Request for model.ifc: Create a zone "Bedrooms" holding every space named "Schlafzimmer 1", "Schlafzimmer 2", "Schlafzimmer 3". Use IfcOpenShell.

First a look at what the model holds.

```python
import ifcopenshell

model = ifcopenshell.open("model.ifc")
print(model.schema)
seen = {}
for space in model.by_type("IfcSpace"):
    seen[space.LongName] = seen.get(space.LongName, 0) + 1
for name, count in sorted(seen.items(), key=str):
    print(count, "x", name)
print("zones:", [z.Name for z in model.by_type("IfcZone")][:20])
```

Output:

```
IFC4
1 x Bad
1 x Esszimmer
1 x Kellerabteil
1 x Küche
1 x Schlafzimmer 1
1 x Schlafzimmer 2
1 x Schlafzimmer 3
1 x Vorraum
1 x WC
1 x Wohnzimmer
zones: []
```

```python
import ifcopenshell
import ifcopenshell.api.group
import ifcopenshell.api.root

model = ifcopenshell.open("model.ifc")

names = {"Schlafzimmer 1", "Schlafzimmer 2", "Schlafzimmer 3"}
spaces = [s for s in model.by_type("IfcSpace") if s.LongName in names]

zone = ifcopenshell.api.root.create_entity(model, ifc_class="IfcZone", name="Bedrooms")
ifcopenshell.api.group.assign_group(model, products=spaces, group=zone)
print(len(spaces), "spaces in", zone.Name)

model.write("model_rev.ifc")
```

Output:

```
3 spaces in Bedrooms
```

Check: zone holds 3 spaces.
